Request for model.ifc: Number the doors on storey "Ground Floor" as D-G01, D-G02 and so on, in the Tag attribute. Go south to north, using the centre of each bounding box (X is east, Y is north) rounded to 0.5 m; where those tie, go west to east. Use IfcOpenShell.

First a look at what the model holds.

```python
import ifcopenshell
import ifcopenshell.util.element
import ifcopenshell.util.placement

model = ifcopenshell.open("model.ifc")
print(model.schema)
storey = next(s for s in model.by_type("IfcBuildingStorey") if s.Name == "Ground Floor")
doors = [e for e in ifcopenshell.util.element.get_decomposition(storey) if e.is_a("IfcDoor")]
for e in sorted(doors, key=lambda e: e.id()):
    origin = ifcopenshell.util.placement.get_local_placement(e.ObjectPlacement)[:3, 3]
    print(e.id(), e.Tag, e.Name, origin.round(2) + 0.0, sep=" | ")
```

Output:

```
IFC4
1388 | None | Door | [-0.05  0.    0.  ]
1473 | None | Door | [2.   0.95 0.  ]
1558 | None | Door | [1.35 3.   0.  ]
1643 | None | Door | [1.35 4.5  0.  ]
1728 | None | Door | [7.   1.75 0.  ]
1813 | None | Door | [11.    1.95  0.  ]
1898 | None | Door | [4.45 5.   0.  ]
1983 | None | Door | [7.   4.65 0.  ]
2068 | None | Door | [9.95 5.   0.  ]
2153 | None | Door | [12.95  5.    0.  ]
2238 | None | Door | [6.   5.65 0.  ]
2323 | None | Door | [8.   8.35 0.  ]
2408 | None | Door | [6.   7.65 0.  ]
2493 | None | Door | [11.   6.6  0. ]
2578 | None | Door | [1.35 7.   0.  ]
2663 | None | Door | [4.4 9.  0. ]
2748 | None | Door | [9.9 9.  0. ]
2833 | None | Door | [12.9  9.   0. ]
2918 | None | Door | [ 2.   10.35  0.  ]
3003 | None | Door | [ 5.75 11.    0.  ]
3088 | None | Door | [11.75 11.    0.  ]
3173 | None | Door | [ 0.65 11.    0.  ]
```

```python
import ifcopenshell
import ifcopenshell.geom
import ifcopenshell.util.element
import ifcopenshell.util.shape

model = ifcopenshell.open("model.ifc")
settings = ifcopenshell.geom.settings()
settings.set("use-world-coords", True)


def centre(element):
    shape = ifcopenshell.geom.create_shape(settings, element)
    return ifcopenshell.util.shape.get_bbox_centroid(shape.geometry)


storey = next(s for s in model.by_type("IfcBuildingStorey") if s.Name == "Ground Floor")
doors = [e for e in ifcopenshell.util.element.get_decomposition(storey) if e.is_a("IfcDoor")]

# Insertion points can sit at a corner or the storey origin, so sort by the geometry (in metres).
centres = {e: centre(e) for e in doors}
doors.sort(key=lambda e: (round(centres[e][1] / 0.5), centres[e][0]))

for i, e in enumerate(doors, start=1):
    number = f"D-G{i:02d}"
    e.Tag = number
    print(e.id(), number)

model.write("model_updated.ifc")
```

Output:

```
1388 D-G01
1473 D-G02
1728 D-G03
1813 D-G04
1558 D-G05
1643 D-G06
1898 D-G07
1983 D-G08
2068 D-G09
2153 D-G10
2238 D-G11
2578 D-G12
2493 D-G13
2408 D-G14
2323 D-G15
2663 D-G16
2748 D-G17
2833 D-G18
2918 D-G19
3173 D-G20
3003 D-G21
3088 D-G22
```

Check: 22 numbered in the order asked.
